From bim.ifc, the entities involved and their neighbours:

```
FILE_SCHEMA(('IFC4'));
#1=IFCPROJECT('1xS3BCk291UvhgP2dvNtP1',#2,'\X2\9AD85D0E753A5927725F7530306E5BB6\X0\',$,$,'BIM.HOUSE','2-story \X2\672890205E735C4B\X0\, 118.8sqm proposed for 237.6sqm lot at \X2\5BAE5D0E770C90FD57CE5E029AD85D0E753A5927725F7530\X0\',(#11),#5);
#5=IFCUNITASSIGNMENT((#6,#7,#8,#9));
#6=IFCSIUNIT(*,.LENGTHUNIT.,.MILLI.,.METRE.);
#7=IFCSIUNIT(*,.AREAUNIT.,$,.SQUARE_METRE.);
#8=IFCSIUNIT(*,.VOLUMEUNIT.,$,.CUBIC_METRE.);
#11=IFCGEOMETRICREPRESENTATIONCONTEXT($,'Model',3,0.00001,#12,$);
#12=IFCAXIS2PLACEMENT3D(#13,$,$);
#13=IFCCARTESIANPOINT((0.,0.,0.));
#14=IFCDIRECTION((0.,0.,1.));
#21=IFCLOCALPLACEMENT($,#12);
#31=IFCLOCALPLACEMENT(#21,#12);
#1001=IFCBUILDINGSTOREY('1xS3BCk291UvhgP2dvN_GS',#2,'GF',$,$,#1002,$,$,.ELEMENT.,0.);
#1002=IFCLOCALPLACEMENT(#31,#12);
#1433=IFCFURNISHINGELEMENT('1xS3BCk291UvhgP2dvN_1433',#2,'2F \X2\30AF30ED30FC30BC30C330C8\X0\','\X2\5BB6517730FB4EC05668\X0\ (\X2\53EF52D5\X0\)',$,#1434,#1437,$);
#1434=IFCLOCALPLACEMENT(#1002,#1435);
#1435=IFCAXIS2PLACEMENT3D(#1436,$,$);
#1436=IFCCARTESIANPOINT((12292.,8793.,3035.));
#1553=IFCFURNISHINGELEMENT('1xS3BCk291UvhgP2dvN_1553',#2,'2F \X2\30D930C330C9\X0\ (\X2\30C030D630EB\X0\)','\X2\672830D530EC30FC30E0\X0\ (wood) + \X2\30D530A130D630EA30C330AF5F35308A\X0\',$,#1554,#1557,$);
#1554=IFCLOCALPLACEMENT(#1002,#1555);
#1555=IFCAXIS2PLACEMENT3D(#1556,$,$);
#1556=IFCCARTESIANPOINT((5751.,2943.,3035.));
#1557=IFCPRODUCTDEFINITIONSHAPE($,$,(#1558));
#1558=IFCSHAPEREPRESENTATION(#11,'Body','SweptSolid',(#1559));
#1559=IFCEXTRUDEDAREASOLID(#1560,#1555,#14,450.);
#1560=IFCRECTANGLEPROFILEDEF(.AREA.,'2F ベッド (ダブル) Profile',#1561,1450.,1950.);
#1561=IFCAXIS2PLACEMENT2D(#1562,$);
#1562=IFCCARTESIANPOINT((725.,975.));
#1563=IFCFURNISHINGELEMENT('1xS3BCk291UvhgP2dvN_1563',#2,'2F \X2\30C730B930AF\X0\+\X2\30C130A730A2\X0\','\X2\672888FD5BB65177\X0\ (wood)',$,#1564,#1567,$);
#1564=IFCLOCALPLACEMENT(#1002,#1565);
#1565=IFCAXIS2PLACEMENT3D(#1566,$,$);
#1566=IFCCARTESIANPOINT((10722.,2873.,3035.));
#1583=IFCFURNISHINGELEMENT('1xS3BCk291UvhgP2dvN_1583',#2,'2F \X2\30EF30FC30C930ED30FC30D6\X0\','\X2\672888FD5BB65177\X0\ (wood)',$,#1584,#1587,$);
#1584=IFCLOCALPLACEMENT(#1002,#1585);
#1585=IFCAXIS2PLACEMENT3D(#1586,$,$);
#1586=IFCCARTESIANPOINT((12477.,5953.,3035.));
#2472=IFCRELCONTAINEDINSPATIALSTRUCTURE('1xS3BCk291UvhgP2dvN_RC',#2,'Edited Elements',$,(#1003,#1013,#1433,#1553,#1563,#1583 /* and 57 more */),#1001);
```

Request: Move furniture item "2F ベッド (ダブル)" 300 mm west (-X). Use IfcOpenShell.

```python
import ifcopenshell
import ifcopenshell.api.geometry
import ifcopenshell.util.placement

model = ifcopenshell.open("bim.ifc")

item = model.by_guid("1xS3BCk291UvhgP2dvN_1553")
matrix = ifcopenshell.util.placement.get_local_placement(item.ObjectPlacement)
matrix[0, 3] -= 300.0
ifcopenshell.api.geometry.edit_object_placement(model, product=item, matrix=matrix, is_si=False)

print(ifcopenshell.util.placement.get_local_placement(item.ObjectPlacement).round(3) + 0.0)

model.write("bim_rev.ifc")
```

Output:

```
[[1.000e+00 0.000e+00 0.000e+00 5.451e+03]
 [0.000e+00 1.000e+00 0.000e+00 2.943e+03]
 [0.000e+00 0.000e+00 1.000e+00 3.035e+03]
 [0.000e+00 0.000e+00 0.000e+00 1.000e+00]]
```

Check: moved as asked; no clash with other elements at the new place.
